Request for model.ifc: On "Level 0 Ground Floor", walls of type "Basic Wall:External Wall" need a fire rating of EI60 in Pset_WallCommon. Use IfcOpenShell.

First a look at what the model holds.

```python
import ifcopenshell
import ifcopenshell.util.element

model = ifcopenshell.open("model.ifc")
print(model.schema)
storey = next(s for s in model.by_type("IfcBuildingStorey") if s.Name == "Level 0 Ground Floor")
walls = [e for e in ifcopenshell.util.element.get_decomposition(storey) if e.is_a("IfcWall")]
seen = {}
for e in walls:
    element_type = ifcopenshell.util.element.get_type(e)
    key = (element_type.Name if element_type != e and element_type else None, ifcopenshell.util.element.get_pset(e, "Pset_WallCommon", "FireRating"))
    seen[key] = seen.get(key, 0) + 1
for (name, value), count in sorted(seen.items(), key=str):
    print(count, "x", name, "|", value)
```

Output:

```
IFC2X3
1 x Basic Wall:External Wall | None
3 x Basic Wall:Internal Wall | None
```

```python
import ifcopenshell
import ifcopenshell.api.pset
import ifcopenshell.util.element

model = ifcopenshell.open("model.ifc")

storey = next(s for s in model.by_type("IfcBuildingStorey") if s.Name == "Level 0 Ground Floor")
walls = [e for e in ifcopenshell.util.element.get_decomposition(storey) if e.is_a("IfcWall")]

count = 0
for e in walls:
    element_type = ifcopenshell.util.element.get_type(e)
    if element_type in (None, e) or element_type.Name != "Basic Wall:External Wall":
        continue
    # add_pset returns the element's existing set when there is one.
    pset = ifcopenshell.api.pset.add_pset(model, product=e, name="Pset_WallCommon")
    ifcopenshell.api.pset.edit_pset(model, pset=pset, properties={"FireRating": "EI60"})
    count += 1

print(count, "walls updated")

model.write("model-out.ifc")
```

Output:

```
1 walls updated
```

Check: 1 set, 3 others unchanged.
